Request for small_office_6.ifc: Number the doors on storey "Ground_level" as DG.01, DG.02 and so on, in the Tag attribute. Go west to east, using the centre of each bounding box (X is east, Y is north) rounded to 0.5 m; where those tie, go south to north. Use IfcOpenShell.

First a look at what the model holds.

```python
import ifcopenshell
import ifcopenshell.util.element
import ifcopenshell.util.placement

model = ifcopenshell.open("small_office_6.ifc")
print(model.schema)
storey = next(s for s in model.by_type("IfcBuildingStorey") if s.Name == "Ground_level")
doors = [e for e in ifcopenshell.util.element.get_decomposition(storey) if e.is_a("IfcDoor")]
for e in sorted(doors, key=lambda e: e.id()):
    origin = ifcopenshell.util.placement.get_local_placement(e.ObjectPlacement)[:3, 3]
    print(e.id(), e.Tag, e.Name, origin.round(2) + 0.0, sep=" | ")
```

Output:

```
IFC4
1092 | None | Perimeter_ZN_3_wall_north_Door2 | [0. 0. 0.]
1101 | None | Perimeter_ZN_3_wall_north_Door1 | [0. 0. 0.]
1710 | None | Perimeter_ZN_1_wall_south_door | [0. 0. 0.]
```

```python
import ifcopenshell
import ifcopenshell.geom
import ifcopenshell.util.element
import ifcopenshell.util.shape

model = ifcopenshell.open("small_office_6.ifc")
settings = ifcopenshell.geom.settings()
settings.set("use-world-coords", True)


def centre(element):
    shape = ifcopenshell.geom.create_shape(settings, element)
    return ifcopenshell.util.shape.get_bbox_centroid(shape.geometry)


storey = next(s for s in model.by_type("IfcBuildingStorey") if s.Name == "Ground_level")
doors = [e for e in ifcopenshell.util.element.get_decomposition(storey) if e.is_a("IfcDoor")]

# Insertion points can sit at a corner or the storey origin, so sort by the geometry (in metres).
centres = {e: centre(e) for e in doors}
doors.sort(key=lambda e: (round(centres[e][0] / 0.5), centres[e][1]))

for i, e in enumerate(doors, start=1):
    number = f"DG.{i:02d}"
    e.Tag = number
    print(e.id(), number)

model.write("small_office_6_updated.ifc")
```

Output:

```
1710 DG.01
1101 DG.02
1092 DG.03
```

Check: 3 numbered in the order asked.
